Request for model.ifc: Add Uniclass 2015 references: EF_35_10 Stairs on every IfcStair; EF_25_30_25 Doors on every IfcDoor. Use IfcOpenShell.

First a look at what the model holds.

```python
import ifcopenshell

model = ifcopenshell.open("model.ifc")
print(model.schema)
print("classifications:", [c.Name for c in model.by_type("IfcClassification")])
for ifc_class in ("IfcDoor", "IfcRoof", "IfcStair", "IfcWall", "IfcWindow"):
    print(ifc_class, len(model.by_type(ifc_class)))
```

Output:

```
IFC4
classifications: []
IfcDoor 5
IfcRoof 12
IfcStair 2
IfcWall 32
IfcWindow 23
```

```python
import ifcopenshell
import ifcopenshell.api.classification

model = ifcopenshell.open("model.ifc")

system = ifcopenshell.api.classification.add_classification(model, classification="Uniclass 2015")

codes = {
    "IfcStair": ("EF_35_10", "Stairs"),
    "IfcDoor": ("EF_25_30_25", "Doors"),
}
for ifc_class, (code, name) in codes.items():
    products = model.by_type(ifc_class)
    ifcopenshell.api.classification.add_reference(
        model, products=products, classification=system, identification=code, name=name
    )
    print(code, len(products))

model.write("model_edited.ifc")
```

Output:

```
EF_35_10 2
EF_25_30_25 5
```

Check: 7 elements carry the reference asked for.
